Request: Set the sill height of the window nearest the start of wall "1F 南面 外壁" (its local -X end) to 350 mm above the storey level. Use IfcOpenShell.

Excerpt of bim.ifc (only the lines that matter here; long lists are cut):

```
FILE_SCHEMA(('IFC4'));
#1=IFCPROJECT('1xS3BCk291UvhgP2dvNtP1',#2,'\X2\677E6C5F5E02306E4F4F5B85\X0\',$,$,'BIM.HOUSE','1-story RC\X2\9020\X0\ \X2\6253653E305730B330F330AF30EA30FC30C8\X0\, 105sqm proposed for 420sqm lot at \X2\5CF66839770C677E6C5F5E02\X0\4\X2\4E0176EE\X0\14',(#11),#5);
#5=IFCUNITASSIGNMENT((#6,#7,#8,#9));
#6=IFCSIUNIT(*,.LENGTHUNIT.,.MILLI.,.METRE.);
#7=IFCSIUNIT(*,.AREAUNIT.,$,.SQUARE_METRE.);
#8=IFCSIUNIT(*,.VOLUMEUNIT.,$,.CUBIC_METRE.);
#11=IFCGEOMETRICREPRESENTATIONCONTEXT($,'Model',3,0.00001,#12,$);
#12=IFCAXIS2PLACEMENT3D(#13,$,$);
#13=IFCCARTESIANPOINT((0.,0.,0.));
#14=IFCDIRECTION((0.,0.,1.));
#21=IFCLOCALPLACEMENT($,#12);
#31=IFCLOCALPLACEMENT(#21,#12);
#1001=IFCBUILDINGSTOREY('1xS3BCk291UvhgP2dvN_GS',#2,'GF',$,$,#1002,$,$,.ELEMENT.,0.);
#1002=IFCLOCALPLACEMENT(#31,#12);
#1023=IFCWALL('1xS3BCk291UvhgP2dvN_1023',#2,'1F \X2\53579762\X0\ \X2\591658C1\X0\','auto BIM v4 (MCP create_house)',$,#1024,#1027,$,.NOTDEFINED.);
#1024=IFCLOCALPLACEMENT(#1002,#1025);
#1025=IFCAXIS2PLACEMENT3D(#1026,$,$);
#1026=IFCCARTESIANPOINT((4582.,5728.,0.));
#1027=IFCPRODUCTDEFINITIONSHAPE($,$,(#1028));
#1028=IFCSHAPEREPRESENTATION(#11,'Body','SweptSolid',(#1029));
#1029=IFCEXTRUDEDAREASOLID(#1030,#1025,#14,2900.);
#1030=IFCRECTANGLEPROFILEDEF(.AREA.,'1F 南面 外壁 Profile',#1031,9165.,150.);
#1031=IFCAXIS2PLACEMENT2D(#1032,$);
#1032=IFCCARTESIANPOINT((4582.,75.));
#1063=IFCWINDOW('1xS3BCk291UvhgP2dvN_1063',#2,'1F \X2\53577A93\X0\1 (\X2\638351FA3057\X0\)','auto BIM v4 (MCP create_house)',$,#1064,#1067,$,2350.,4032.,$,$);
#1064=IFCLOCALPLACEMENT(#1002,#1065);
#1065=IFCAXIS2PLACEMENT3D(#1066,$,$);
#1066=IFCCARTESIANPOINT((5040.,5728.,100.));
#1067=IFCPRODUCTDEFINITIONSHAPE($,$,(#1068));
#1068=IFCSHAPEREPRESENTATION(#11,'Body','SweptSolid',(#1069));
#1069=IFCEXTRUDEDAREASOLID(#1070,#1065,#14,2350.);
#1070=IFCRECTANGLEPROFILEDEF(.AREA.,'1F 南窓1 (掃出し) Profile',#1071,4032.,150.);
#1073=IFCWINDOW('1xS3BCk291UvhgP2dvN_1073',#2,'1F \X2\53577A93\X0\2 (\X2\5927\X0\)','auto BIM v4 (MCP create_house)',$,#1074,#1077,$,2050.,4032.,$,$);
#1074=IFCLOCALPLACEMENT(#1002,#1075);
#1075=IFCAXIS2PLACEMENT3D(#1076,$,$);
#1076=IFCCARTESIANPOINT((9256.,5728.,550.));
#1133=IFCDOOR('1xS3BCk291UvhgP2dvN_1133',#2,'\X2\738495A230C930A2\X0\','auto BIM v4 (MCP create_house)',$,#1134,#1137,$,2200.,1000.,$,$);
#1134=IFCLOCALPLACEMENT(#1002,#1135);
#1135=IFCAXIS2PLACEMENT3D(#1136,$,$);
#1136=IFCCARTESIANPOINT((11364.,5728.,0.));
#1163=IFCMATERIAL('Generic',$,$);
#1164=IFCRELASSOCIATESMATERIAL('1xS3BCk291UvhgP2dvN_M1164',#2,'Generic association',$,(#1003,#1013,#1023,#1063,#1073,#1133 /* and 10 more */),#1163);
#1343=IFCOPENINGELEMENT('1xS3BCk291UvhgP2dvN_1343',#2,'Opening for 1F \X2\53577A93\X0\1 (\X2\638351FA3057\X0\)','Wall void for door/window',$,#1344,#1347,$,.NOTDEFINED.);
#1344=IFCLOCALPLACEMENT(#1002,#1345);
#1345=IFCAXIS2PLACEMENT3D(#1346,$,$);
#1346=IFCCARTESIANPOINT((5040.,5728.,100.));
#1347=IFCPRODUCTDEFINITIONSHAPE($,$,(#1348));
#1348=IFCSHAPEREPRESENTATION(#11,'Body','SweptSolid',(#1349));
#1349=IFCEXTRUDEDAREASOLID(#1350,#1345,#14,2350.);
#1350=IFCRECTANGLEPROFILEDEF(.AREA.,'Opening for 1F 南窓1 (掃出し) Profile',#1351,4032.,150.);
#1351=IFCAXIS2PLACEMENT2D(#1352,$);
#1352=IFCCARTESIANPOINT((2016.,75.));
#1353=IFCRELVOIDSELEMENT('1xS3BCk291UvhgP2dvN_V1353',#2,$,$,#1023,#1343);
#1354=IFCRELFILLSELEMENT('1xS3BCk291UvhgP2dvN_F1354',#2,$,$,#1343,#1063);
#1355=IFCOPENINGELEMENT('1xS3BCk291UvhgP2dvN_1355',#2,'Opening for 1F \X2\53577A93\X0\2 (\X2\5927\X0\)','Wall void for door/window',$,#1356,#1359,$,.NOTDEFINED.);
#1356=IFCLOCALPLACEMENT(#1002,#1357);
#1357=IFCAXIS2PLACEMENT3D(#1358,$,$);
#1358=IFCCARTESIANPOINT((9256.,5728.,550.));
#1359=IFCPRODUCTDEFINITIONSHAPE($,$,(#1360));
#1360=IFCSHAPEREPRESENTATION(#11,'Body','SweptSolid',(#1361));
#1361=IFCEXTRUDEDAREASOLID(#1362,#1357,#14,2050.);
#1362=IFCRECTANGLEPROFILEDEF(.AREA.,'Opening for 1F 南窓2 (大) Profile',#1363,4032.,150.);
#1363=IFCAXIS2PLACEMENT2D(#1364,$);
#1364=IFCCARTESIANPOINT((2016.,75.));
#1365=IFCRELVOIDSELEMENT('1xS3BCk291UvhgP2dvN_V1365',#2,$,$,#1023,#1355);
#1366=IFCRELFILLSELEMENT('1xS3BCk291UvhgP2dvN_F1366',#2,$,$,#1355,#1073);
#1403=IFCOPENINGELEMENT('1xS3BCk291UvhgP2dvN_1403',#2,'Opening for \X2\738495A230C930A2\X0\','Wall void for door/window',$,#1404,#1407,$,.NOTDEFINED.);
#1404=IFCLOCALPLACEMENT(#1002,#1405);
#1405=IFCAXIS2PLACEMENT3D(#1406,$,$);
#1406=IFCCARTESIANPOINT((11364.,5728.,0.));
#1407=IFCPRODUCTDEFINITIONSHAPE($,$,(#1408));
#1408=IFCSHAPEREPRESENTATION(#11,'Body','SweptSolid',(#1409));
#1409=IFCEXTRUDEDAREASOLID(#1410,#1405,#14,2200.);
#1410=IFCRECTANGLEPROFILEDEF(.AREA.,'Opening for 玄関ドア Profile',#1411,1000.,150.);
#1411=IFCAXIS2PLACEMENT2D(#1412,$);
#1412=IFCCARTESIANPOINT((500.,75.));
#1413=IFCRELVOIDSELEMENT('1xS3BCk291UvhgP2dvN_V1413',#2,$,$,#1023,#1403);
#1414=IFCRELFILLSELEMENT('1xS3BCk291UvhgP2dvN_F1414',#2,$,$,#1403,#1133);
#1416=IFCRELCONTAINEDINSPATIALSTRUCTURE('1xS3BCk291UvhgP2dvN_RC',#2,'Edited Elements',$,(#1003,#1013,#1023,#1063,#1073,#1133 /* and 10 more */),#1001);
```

```python
import numpy as np
import ifcopenshell
import ifcopenshell.api.geometry
import ifcopenshell.geom
import ifcopenshell.util.element
import ifcopenshell.util.placement
import ifcopenshell.util.shape
import ifcopenshell.util.unit

model = ifcopenshell.open("bim.ifc")
unit_scale = ifcopenshell.util.unit.calculate_unit_scale(model)

window = model.by_guid("1xS3BCk291UvhgP2dvN_1063")
opening = window.FillsVoids[0].RelatingOpeningElement
storey = ifcopenshell.util.element.get_container(window, ifc_class="IfcBuildingStorey")
level = ifcopenshell.util.placement.get_local_placement(storey.ObjectPlacement)[2, 3]

# The opening's origin need not be at the sill, so measure its lowest point.
shape = ifcopenshell.geom.create_shape(ifcopenshell.geom.settings(), opening)
bottom = ifcopenshell.util.shape.get_shape_bottom_elevation(shape, shape.geometry) / unit_scale
dz = level + 0.35 / unit_scale - bottom

shift = np.array([0.0, 0.0, dz])
# The window is not placed relative to its opening, so move both.
for product in (opening, window):
    matrix = ifcopenshell.util.placement.get_local_placement(product.ObjectPlacement)
    matrix[:3, 3] += shift
    ifcopenshell.api.geometry.edit_object_placement(model, product=product, matrix=matrix, is_si=False)

print(f"moved by {dz * unit_scale:+.3f} m")

model.write("bim_v2.ifc")
```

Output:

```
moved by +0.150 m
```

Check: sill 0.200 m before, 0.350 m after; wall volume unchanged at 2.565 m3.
